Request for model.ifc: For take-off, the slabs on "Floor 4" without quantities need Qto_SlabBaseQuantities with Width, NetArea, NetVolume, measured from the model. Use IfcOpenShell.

First a look at what the model holds.

```python
import ifcopenshell
import ifcopenshell.util.element
import ifcopenshell.util.unit

model = ifcopenshell.open("model.ifc")
print(model.schema)
for unit_type in ("LENGTHUNIT", "AREAUNIT", "VOLUMEUNIT"):
    print(unit_type, ifcopenshell.util.unit.calculate_unit_scale(model, unit_type))
storey = next(s for s in model.by_type("IfcBuildingStorey") if s.Name == "Floor 4")
slabs = [e for e in ifcopenshell.util.element.get_decomposition(storey) if e.is_a("IfcSlab")]
for e in sorted(slabs, key=lambda e: e.id()):
    print(e.id(), e.is_a(), e.Name, list(ifcopenshell.util.element.get_psets(e, qtos_only=True)), sep=" | ")
```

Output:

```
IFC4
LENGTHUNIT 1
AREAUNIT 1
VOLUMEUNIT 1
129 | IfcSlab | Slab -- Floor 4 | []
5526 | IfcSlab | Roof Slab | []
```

```python
import ifcopenshell
import ifcopenshell.api.pset
import ifcopenshell.geom
import ifcopenshell.util.element
import ifcopenshell.util.shape
import ifcopenshell.util.unit

model = ifcopenshell.open("model.ifc")
unit_scale = ifcopenshell.util.unit.calculate_unit_scale(model)
area_scale = ifcopenshell.util.unit.calculate_unit_scale(model, "AREAUNIT")
volume_scale = ifcopenshell.util.unit.calculate_unit_scale(model, "VOLUMEUNIT")
settings = ifcopenshell.geom.settings()

storey = next(s for s in model.by_type("IfcBuildingStorey") if s.Name == "Floor 4")
slabs = [e for e in ifcopenshell.util.element.get_decomposition(storey) if e.is_a("IfcSlab")]

for e in sorted(slabs, key=lambda e: e.id()):
    if ifcopenshell.util.element.get_psets(e, qtos_only=True, should_inherit=False):
        continue
    # Geometry comes back in metres, in the element's own axes.
    shape = ifcopenshell.geom.create_shape(settings, e)
    values = {
        "Width": ifcopenshell.util.shape.get_z(shape.geometry) / unit_scale,
        "NetArea": ifcopenshell.util.shape.get_footprint_area(shape.geometry) / area_scale,
        "NetVolume": ifcopenshell.util.shape.get_volume(shape.geometry) / volume_scale,
    }
    qto = ifcopenshell.api.pset.add_qto(model, product=e, name="Qto_SlabBaseQuantities")
    ifcopenshell.api.pset.edit_qto(model, qto=qto, properties=values)
    print(e.id(), {k: round(v, 3) for k, v in values.items()})

model.write("model_edited.ifc")
```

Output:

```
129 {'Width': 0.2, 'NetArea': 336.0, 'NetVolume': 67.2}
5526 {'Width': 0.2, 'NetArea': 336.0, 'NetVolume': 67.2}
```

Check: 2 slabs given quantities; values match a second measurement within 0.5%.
